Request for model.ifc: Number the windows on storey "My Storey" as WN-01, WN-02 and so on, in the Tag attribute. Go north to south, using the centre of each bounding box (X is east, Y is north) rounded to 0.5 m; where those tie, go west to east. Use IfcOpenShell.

First a look at what the model holds.

```python
import ifcopenshell
import ifcopenshell.util.element
import ifcopenshell.util.placement

model = ifcopenshell.open("model.ifc")
print(model.schema)
storey = next(s for s in model.by_type("IfcBuildingStorey") if s.Name == "My Storey")
windows = [e for e in ifcopenshell.util.element.get_decomposition(storey) if e.is_a("IfcWindow")]
for e in sorted(windows, key=lambda e: e.id()):
    origin = ifcopenshell.util.placement.get_local_placement(e.ObjectPlacement)[:3, 3]
    print(e.id(), e.Tag, e.Name, origin.round(2) + 0.0, sep=" | ")
```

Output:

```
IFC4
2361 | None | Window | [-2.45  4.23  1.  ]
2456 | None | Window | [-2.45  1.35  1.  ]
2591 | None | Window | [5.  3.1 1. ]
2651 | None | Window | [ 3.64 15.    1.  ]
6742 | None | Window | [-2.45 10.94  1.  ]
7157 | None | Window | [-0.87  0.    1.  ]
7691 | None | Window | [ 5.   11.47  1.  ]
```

```python
import ifcopenshell
import ifcopenshell.geom
import ifcopenshell.util.element
import ifcopenshell.util.shape

model = ifcopenshell.open("model.ifc")
settings = ifcopenshell.geom.settings()
settings.set("use-world-coords", True)


def centre(element):
    shape = ifcopenshell.geom.create_shape(settings, element)
    return ifcopenshell.util.shape.get_bbox_centroid(shape.geometry)


storey = next(s for s in model.by_type("IfcBuildingStorey") if s.Name == "My Storey")
windows = [e for e in ifcopenshell.util.element.get_decomposition(storey) if e.is_a("IfcWindow")]

# Insertion points can sit at a corner or the storey origin, so sort by the geometry (in metres).
centres = {e: centre(e) for e in windows}
windows.sort(key=lambda e: (-round(centres[e][1] / 0.5), centres[e][0]))

for i, e in enumerate(windows, start=1):
    number = f"WN-{i:02d}"
    e.Tag = number
    print(e.id(), number)

model.write("model_edited.ifc")
```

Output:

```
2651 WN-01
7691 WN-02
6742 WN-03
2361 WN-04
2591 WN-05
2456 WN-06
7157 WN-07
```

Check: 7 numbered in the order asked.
